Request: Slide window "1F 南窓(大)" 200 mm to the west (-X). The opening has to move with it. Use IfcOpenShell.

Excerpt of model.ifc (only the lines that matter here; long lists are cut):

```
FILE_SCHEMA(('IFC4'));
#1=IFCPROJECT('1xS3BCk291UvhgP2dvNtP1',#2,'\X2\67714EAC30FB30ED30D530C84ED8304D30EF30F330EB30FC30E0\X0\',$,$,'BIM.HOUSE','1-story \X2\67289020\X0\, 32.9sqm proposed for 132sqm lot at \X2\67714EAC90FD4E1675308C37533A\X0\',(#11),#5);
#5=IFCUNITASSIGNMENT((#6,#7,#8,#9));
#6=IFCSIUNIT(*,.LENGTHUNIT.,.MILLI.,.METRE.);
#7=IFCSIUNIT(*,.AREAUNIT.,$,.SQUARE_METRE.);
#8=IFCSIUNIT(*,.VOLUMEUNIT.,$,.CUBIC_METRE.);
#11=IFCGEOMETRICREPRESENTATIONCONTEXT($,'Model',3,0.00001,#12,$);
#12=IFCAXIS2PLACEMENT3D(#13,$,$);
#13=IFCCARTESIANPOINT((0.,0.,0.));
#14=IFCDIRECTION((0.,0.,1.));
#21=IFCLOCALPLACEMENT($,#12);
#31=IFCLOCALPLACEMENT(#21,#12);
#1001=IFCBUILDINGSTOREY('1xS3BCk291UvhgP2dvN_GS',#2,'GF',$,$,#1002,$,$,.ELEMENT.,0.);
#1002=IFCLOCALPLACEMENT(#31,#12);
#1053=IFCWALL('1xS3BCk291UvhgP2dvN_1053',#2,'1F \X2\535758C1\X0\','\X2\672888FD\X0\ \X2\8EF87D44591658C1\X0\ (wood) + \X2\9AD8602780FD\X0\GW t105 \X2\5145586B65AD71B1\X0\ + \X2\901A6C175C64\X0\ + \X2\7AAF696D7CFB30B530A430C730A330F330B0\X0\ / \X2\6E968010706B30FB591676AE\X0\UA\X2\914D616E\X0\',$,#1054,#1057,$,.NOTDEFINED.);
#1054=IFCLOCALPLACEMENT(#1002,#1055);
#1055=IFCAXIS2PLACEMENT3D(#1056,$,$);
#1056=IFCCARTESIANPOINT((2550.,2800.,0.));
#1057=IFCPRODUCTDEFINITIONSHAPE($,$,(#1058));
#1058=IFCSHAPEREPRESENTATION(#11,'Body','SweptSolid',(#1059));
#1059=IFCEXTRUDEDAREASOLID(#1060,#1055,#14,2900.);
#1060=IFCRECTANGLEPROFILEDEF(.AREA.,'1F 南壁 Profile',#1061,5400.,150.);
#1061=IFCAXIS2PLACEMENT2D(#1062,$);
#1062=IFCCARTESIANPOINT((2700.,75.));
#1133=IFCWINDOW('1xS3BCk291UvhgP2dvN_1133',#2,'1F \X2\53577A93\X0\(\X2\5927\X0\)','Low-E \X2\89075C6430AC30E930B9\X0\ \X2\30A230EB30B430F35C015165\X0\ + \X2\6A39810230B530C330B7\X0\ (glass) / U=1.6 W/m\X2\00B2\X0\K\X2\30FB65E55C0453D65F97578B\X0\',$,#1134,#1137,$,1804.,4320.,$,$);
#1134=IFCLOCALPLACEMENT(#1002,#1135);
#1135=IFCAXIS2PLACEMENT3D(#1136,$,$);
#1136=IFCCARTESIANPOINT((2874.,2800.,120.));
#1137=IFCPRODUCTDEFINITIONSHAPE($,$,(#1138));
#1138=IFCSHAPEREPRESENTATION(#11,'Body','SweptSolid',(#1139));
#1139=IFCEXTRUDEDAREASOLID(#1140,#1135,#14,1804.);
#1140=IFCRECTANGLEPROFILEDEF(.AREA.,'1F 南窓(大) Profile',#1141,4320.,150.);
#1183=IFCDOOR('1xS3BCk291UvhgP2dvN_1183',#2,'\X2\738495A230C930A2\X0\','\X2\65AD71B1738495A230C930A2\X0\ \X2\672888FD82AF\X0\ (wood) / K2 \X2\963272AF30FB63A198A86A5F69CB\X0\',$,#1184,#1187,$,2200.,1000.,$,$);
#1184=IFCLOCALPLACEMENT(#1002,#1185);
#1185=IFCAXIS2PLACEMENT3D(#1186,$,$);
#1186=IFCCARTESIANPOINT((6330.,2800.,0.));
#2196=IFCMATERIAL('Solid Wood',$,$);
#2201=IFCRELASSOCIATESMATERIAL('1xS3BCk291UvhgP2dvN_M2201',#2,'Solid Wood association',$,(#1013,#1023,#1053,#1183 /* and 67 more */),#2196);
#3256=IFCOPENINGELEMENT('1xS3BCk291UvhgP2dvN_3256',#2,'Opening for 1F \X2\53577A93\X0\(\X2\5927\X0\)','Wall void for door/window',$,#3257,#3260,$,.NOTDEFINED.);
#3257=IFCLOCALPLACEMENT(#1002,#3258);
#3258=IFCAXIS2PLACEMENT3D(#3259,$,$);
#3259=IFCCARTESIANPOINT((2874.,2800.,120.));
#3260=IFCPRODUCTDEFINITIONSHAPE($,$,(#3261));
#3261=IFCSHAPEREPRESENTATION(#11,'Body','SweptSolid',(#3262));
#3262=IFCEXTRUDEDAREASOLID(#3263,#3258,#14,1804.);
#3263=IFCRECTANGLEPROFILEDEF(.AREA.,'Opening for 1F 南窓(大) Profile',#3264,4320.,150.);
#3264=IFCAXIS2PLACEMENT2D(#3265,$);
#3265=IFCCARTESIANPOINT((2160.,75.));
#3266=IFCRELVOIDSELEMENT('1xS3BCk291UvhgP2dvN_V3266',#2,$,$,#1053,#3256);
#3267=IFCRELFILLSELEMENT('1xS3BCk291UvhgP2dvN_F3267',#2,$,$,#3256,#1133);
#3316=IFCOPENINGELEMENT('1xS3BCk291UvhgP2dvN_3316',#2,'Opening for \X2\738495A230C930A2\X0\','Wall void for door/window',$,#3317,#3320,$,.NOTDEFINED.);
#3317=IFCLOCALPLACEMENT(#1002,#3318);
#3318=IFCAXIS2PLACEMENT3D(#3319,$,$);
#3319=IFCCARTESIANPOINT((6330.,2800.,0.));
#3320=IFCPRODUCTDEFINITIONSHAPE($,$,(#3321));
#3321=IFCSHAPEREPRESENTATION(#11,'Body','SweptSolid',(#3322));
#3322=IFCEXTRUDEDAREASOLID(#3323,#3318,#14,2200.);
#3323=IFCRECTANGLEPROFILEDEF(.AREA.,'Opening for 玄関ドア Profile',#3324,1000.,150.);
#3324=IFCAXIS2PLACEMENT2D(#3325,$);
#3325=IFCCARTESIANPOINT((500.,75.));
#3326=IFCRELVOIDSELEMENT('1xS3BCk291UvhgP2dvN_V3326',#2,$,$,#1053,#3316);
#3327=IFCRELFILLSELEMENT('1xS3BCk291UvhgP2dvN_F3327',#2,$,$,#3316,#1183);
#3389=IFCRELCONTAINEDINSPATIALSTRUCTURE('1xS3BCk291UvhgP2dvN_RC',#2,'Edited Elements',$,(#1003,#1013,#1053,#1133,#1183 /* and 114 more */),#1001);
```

```python
import ifcopenshell
import ifcopenshell.api.geometry
import ifcopenshell.util.placement
import ifcopenshell.util.unit

model = ifcopenshell.open("model.ifc")
unit_scale = ifcopenshell.util.unit.calculate_unit_scale(model)

window = model.by_guid("1xS3BCk291UvhgP2dvN_1133")
opening = window.FillsVoids[0].RelatingOpeningElement
wall = opening.VoidsElements[0].RelatingBuildingElement

wall_matrix = ifcopenshell.util.placement.get_local_placement(wall.ObjectPlacement)
shift = wall_matrix[:3, 0] * -0.2 / unit_scale
before = ifcopenshell.util.placement.get_local_placement(window.ObjectPlacement)[:3, 3].copy()

# The window is not placed relative to its opening, so move both.
for product in (opening, window):
    matrix = ifcopenshell.util.placement.get_local_placement(product.ObjectPlacement)
    matrix[:3, 3] += shift
    ifcopenshell.api.geometry.edit_object_placement(model, product=product, matrix=matrix, is_si=False)

after = ifcopenshell.util.placement.get_local_placement(window.ObjectPlacement)[:3, 3]
print("window moved by", (after - before).round(3) + 0.0)

model.write("model-out.ifc")
```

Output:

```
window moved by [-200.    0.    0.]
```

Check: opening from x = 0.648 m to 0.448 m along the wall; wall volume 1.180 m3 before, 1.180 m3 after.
